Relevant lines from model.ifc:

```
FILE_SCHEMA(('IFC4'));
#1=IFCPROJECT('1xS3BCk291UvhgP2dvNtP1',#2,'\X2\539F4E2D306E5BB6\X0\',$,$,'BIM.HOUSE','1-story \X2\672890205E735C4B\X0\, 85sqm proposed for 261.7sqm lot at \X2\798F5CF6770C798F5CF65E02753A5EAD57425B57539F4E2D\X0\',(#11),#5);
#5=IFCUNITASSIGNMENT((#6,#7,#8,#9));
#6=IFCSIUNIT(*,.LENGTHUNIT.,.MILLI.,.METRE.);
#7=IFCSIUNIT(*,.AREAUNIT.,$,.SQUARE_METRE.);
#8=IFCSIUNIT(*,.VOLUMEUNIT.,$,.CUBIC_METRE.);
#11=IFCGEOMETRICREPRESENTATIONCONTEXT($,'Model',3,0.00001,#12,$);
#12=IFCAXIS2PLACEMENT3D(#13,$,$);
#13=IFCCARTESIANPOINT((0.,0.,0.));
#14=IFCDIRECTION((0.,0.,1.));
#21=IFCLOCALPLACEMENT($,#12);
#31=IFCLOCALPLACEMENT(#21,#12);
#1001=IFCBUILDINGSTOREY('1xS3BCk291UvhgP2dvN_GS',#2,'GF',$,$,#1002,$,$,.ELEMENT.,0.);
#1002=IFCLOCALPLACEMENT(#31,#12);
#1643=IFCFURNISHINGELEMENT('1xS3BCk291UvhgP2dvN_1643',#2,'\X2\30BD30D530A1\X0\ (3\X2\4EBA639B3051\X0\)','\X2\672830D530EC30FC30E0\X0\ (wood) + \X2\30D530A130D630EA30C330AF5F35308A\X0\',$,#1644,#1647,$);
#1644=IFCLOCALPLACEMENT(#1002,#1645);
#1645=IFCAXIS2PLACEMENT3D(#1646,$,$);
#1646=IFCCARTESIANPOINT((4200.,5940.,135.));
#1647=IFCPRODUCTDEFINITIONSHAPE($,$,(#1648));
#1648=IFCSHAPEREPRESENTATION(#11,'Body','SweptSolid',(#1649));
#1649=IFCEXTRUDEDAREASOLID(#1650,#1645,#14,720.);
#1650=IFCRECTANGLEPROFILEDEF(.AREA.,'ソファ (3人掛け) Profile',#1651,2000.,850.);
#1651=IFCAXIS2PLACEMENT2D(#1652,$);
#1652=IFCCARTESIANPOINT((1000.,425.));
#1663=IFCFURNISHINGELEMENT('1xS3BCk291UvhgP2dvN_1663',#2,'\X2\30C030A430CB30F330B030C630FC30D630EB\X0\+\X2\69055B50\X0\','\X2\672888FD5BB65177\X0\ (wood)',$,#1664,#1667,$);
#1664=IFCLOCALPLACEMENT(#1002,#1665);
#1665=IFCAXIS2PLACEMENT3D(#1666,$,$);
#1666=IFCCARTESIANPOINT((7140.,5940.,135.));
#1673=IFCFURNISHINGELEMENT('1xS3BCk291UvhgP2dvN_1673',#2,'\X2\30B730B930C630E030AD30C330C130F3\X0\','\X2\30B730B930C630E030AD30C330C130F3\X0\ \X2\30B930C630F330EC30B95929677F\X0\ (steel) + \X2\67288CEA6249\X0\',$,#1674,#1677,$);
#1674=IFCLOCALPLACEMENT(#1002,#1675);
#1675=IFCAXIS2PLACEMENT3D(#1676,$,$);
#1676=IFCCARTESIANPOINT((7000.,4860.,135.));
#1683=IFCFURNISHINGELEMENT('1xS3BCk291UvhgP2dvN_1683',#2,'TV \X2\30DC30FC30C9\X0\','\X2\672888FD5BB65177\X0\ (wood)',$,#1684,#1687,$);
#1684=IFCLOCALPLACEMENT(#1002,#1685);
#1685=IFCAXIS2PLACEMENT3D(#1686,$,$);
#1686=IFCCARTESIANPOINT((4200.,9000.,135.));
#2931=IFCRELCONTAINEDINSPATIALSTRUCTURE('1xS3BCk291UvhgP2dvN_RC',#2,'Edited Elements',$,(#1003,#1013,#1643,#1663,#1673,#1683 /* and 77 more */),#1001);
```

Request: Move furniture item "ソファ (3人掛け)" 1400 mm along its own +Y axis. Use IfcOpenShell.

```python
import ifcopenshell
import ifcopenshell.api.geometry
import ifcopenshell.util.placement
import ifcopenshell.util.unit

model = ifcopenshell.open("model.ifc")
unit_scale = ifcopenshell.util.unit.calculate_unit_scale(model)

item = model.by_guid("1xS3BCk291UvhgP2dvN_1643")
matrix = ifcopenshell.util.placement.get_local_placement(item.ObjectPlacement)
matrix[:3, 3] += matrix[:3, 1] * 1.4 / unit_scale
ifcopenshell.api.geometry.edit_object_placement(model, product=item, matrix=matrix, is_si=False)

print(ifcopenshell.util.placement.get_local_placement(item.ObjectPlacement).round(3) + 0.0)

model.write("model_updated.ifc")
```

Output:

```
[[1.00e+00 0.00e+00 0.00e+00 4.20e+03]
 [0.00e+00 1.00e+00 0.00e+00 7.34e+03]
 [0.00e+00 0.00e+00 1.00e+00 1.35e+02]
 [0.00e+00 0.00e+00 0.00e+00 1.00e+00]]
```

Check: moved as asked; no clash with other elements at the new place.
